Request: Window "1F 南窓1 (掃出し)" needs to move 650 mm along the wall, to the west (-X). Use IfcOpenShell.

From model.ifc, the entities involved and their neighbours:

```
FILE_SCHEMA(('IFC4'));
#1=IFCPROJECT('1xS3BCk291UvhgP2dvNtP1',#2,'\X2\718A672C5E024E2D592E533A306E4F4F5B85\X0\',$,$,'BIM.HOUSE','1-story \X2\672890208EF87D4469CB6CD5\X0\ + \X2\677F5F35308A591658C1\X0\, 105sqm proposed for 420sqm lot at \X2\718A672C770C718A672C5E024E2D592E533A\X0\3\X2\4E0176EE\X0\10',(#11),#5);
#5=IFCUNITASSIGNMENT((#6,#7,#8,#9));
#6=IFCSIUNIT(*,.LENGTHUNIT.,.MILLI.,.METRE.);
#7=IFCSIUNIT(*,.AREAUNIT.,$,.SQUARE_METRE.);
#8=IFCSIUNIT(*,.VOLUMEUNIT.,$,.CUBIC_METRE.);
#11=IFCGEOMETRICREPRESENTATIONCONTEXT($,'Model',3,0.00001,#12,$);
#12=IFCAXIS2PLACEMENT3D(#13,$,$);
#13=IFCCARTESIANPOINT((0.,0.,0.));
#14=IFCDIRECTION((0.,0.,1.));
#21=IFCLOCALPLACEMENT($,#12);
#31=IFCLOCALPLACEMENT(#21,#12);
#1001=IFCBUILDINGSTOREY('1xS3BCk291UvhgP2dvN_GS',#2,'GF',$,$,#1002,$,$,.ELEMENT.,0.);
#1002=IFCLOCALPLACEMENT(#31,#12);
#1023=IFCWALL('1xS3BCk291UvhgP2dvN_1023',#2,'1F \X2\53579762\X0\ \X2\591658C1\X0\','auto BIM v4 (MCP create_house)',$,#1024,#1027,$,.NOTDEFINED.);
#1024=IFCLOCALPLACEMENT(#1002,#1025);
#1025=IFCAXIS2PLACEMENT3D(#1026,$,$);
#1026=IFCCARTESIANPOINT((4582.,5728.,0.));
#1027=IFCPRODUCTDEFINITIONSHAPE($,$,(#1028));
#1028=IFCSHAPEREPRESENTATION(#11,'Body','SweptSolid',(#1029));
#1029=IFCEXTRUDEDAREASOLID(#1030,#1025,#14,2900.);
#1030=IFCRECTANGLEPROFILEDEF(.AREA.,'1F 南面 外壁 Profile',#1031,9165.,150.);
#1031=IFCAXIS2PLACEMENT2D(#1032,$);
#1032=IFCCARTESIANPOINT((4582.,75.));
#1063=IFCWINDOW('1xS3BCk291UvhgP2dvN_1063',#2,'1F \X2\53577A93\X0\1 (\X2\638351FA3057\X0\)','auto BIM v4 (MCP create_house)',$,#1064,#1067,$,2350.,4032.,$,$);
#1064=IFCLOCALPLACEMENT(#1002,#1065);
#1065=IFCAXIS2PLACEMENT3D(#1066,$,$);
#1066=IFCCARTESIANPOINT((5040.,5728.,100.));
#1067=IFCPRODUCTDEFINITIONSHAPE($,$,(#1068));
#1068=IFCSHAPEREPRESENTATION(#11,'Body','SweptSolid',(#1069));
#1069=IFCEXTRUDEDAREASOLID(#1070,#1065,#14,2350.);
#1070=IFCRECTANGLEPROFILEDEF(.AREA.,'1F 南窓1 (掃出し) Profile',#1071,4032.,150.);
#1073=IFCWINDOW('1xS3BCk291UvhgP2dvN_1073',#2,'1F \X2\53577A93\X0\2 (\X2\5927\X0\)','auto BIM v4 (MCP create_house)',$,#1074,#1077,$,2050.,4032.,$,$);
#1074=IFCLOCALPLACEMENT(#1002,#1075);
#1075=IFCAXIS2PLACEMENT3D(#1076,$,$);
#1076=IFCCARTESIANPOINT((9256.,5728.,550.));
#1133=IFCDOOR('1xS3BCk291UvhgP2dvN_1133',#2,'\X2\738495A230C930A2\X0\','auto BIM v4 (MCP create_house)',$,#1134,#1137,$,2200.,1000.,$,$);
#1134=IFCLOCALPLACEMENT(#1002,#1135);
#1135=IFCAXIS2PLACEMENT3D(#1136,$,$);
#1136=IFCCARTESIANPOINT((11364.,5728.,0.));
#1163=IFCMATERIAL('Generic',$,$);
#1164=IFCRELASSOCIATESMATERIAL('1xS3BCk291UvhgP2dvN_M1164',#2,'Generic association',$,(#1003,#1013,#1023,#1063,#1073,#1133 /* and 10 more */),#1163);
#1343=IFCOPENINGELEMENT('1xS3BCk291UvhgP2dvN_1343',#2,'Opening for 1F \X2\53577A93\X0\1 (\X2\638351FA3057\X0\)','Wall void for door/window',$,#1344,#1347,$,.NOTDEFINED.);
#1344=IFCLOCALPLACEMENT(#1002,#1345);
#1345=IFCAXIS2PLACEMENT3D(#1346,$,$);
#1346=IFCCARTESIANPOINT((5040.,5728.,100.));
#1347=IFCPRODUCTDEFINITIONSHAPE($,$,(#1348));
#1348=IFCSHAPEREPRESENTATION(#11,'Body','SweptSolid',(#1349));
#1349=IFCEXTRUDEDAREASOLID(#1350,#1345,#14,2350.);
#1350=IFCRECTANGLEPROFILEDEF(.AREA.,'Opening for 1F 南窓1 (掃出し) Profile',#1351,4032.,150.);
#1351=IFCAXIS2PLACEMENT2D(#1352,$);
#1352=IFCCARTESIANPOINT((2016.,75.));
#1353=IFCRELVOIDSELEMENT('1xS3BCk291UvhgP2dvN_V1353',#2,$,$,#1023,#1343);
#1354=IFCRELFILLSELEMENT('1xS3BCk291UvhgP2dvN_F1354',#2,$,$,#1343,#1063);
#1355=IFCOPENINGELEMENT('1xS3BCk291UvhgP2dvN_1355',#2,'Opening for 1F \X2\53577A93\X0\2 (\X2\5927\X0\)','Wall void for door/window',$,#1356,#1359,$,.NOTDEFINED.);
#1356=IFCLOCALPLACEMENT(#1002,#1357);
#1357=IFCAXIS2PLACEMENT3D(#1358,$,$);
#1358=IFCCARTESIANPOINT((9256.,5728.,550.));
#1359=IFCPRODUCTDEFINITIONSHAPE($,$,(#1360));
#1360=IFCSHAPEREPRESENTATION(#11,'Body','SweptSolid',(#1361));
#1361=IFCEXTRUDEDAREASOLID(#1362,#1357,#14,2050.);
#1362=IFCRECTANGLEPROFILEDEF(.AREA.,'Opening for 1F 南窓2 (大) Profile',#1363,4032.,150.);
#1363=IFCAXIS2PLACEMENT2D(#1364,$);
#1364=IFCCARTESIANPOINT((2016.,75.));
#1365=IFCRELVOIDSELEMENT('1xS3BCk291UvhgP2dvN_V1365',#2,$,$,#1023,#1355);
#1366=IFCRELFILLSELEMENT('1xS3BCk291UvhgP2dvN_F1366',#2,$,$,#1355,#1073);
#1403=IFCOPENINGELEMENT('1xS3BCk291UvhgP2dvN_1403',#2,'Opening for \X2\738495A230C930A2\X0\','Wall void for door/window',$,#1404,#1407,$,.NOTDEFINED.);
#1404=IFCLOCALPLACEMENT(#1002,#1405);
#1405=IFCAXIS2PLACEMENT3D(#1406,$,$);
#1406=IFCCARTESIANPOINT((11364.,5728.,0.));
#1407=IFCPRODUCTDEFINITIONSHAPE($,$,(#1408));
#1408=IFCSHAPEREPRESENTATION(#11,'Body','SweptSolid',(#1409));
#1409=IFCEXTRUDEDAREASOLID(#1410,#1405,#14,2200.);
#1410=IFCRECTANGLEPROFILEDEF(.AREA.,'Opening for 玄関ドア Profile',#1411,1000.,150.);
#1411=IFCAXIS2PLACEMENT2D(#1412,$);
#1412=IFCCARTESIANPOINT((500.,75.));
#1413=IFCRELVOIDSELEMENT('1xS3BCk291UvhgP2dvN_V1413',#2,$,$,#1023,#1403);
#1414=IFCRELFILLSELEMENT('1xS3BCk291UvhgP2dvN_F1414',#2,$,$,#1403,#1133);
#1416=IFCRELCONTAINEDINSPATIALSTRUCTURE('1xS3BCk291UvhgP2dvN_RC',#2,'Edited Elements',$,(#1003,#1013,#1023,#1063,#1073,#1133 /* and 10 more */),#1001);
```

```python
import ifcopenshell
import ifcopenshell.api.geometry
import ifcopenshell.util.placement

model = ifcopenshell.open("model.ifc")

window = model.by_guid("1xS3BCk291UvhgP2dvN_1063")
opening = window.FillsVoids[0].RelatingOpeningElement
wall = opening.VoidsElements[0].RelatingBuildingElement

wall_matrix = ifcopenshell.util.placement.get_local_placement(wall.ObjectPlacement)
shift = wall_matrix[:3, 0] * -650.0
before = ifcopenshell.util.placement.get_local_placement(window.ObjectPlacement)[:3, 3].copy()

# The window is not placed relative to its opening, so move both.
for product in (opening, window):
    matrix = ifcopenshell.util.placement.get_local_placement(product.ObjectPlacement)
    matrix[:3, 3] += shift
    ifcopenshell.api.geometry.edit_object_placement(model, product=product, matrix=matrix, is_si=False)

after = ifcopenshell.util.placement.get_local_placement(window.ObjectPlacement)[:3, 3]
print("window moved by", (after - before).round(3) + 0.0)

model.write("model_updated.ifc")
```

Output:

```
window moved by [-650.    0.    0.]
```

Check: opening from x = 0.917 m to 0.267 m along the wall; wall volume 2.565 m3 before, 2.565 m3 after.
